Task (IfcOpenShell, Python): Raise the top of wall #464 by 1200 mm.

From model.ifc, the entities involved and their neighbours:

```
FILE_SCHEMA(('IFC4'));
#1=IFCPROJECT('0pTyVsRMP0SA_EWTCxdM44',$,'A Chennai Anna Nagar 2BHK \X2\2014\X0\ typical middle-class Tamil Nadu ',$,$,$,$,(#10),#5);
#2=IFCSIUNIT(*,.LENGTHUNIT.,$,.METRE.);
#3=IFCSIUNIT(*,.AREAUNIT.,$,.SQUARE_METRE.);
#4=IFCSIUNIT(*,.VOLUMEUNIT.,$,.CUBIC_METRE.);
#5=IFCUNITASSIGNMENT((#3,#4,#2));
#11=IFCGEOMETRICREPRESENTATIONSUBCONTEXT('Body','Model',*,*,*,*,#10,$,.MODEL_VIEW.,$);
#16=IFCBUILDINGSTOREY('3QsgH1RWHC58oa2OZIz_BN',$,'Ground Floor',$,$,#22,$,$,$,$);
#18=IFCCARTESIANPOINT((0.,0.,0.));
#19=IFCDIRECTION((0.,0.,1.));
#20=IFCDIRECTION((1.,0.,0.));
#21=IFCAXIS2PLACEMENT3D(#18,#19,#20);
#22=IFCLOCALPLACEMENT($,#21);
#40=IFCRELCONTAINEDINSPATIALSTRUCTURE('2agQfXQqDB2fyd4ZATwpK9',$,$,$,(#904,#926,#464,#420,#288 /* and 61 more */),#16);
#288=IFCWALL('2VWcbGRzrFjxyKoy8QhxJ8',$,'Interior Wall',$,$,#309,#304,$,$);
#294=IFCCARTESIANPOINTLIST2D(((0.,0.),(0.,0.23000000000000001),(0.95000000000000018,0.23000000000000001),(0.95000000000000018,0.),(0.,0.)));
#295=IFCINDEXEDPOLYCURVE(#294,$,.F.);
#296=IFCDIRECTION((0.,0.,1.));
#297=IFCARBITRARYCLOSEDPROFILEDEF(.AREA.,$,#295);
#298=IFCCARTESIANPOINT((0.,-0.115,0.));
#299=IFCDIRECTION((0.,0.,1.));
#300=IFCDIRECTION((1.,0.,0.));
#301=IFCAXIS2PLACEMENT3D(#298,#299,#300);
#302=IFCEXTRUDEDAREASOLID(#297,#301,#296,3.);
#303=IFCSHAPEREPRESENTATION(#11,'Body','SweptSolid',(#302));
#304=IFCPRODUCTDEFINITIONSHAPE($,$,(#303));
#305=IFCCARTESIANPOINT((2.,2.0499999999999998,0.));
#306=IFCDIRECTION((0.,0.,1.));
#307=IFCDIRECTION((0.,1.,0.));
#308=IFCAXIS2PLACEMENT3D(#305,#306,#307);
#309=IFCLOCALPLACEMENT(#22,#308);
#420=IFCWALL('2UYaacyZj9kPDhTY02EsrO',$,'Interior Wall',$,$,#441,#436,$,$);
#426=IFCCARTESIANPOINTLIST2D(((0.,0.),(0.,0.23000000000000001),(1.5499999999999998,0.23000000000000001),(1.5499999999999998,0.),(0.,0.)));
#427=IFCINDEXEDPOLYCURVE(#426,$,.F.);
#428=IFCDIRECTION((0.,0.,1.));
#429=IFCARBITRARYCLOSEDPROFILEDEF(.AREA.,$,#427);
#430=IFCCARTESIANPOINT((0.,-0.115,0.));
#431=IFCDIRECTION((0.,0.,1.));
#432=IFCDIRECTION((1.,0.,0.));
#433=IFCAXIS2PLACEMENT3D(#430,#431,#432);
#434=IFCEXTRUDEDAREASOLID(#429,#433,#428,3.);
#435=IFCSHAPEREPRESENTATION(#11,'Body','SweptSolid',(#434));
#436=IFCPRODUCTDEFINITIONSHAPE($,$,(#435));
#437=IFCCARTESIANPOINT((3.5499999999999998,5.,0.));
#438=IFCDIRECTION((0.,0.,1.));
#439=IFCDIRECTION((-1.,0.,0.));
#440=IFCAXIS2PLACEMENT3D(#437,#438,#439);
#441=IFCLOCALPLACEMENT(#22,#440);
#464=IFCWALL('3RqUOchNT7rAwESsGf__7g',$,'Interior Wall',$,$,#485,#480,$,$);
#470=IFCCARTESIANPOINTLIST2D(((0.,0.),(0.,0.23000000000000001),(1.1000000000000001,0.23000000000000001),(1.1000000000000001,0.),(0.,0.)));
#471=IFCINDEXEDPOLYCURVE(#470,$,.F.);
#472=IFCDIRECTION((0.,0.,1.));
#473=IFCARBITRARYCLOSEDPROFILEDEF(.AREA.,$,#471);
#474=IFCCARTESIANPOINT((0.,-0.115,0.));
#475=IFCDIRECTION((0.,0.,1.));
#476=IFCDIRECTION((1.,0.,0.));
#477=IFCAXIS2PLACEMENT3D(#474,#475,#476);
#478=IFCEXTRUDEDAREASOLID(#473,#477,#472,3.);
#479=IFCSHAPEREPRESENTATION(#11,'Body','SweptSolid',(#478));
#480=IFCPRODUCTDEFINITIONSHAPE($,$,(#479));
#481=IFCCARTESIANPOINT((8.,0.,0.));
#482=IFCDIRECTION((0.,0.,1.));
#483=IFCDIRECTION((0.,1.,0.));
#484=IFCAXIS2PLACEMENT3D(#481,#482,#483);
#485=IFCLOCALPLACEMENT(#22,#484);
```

```python
import ifcopenshell
import ifcopenshell.geom
import ifcopenshell.util.representation
import ifcopenshell.util.shape
import ifcopenshell.util.unit

model = ifcopenshell.open("model.ifc")
unit_scale = ifcopenshell.util.unit.calculate_unit_scale(model)
settings = ifcopenshell.geom.settings()


def volume(element):
    """Net volume in cubic metres, openings subtracted."""
    shape = ifcopenshell.geom.create_shape(settings, element)
    return ifcopenshell.util.shape.get_volume(shape.geometry)


wall = model.by_id(464)
before = volume(wall)

body = ifcopenshell.util.representation.get_representation(wall, "Model", "Body")
solid = body.Items[0]
old_height = solid.Depth
solid.Depth += 1.2 / unit_scale
after = volume(wall)

print(f"height {old_height:g} -> {solid.Depth:g}, volume {before:.3f} -> {after:.3f} m3")

model.write("model_updated.ifc")
```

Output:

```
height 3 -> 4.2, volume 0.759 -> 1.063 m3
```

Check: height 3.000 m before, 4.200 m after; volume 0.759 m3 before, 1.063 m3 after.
